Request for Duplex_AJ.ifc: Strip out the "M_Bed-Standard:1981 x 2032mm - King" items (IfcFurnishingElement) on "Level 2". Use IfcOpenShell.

First a look at what the model holds.

```python
import ifcopenshell
import ifcopenshell.util.element

model = ifcopenshell.open("Duplex_AJ.ifc")
print(model.schema)
storey = next(s for s in model.by_type("IfcBuildingStorey") if s.Name == "Level 2")
furniture = [e for e in ifcopenshell.util.element.get_decomposition(storey) if e.is_a("IfcFurnishingElement")]
seen = {}
for e in furniture:
    element_type = ifcopenshell.util.element.get_type(e)
    name = element_type.Name if element_type not in (None, e) else None
    seen[name] = seen.get(name, 0) + 1
for name, count in sorted(seen.items(), key=str):
    print(count, "x", name)
```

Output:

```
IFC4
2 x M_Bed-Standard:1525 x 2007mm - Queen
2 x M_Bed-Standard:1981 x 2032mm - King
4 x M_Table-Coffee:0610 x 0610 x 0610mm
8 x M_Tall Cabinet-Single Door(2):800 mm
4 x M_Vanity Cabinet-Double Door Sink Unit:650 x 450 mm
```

```python
import ifcopenshell
import ifcopenshell.api.root
import ifcopenshell.util.element

model = ifcopenshell.open("Duplex_AJ.ifc")

storey = next(s for s in model.by_type("IfcBuildingStorey") if s.Name == "Level 2")
furniture = [e for e in ifcopenshell.util.element.get_decomposition(storey) if e.is_a("IfcFurnishingElement")]
targets = [e for e in furniture if (t := ifcopenshell.util.element.get_type(e)) not in (None, e) and t.Name == "M_Bed-Standard:1981 x 2032mm - King"]

for e in targets:
    ifcopenshell.api.root.remove_product(model, product=e)
print(len(targets), "removed")

model.write("Duplex_AJ_rev.ifc")
```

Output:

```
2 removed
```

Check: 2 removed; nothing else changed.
